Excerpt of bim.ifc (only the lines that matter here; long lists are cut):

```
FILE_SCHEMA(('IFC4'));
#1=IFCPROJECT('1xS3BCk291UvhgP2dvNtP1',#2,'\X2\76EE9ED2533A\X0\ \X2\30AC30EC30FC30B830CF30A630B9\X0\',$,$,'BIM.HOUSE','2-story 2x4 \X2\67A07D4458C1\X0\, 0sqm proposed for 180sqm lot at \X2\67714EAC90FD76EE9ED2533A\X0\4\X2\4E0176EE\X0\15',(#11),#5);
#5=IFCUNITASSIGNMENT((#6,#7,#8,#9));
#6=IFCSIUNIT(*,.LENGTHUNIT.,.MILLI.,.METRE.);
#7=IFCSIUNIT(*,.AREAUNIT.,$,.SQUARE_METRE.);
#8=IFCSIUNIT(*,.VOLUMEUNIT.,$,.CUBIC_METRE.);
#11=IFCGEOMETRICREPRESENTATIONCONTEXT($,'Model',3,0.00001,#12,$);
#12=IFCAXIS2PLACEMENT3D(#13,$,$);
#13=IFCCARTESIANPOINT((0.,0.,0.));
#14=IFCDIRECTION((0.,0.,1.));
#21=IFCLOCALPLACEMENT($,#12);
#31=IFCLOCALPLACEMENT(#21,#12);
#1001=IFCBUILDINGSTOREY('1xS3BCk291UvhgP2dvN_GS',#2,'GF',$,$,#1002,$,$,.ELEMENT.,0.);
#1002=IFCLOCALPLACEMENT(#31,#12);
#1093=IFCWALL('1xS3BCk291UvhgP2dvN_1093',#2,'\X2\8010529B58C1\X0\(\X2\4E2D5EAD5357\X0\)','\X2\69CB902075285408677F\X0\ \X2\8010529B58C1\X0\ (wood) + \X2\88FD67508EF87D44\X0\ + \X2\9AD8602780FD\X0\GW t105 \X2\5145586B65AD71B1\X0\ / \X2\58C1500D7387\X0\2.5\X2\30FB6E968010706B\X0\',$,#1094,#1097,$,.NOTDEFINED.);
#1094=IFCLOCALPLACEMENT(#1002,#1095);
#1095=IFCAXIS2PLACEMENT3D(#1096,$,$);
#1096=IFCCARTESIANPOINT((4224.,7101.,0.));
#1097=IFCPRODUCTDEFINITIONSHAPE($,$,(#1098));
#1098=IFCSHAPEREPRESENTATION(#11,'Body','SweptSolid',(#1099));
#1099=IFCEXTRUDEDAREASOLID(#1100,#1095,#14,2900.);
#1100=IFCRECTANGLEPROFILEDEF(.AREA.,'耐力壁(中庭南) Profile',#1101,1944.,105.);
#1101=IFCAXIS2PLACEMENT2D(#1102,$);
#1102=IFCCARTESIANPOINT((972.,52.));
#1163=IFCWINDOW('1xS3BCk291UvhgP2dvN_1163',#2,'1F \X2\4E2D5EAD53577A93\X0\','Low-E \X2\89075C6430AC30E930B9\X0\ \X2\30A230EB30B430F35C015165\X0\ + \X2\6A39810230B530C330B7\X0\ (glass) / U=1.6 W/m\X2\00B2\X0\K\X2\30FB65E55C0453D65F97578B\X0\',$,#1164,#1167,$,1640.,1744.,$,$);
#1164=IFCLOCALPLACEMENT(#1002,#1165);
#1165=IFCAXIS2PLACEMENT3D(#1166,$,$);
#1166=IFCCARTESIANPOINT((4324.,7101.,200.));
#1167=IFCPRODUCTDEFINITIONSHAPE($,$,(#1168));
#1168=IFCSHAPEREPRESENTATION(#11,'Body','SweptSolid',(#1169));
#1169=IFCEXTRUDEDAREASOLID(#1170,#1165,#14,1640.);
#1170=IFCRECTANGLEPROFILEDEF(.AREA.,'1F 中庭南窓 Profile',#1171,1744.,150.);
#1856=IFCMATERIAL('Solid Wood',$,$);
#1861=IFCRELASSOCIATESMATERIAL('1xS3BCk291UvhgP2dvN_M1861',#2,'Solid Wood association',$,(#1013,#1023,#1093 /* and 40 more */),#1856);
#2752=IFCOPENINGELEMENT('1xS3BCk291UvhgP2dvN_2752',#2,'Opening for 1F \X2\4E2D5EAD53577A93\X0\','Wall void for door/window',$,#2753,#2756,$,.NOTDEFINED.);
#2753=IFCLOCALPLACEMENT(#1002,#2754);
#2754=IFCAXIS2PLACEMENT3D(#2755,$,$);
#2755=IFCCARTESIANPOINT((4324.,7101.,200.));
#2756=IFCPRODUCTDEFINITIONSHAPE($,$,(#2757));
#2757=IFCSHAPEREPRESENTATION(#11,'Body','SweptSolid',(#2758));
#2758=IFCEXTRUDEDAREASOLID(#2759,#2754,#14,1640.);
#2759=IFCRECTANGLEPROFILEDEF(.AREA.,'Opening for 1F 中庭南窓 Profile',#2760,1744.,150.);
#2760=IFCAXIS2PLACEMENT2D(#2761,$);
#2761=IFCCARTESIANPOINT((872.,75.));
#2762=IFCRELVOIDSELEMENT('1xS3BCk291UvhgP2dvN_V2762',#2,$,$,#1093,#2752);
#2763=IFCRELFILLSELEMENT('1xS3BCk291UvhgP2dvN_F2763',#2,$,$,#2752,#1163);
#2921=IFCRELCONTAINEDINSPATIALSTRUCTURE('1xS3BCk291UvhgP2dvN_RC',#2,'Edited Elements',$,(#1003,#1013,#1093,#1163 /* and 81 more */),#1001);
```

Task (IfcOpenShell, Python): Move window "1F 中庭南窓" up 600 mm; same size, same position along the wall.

```python
import numpy as np
import ifcopenshell
import ifcopenshell.api.geometry
import ifcopenshell.util.placement
import ifcopenshell.util.unit

model = ifcopenshell.open("bim.ifc")
unit_scale = ifcopenshell.util.unit.calculate_unit_scale(model)

window = model.by_guid("1xS3BCk291UvhgP2dvN_1163")
opening = window.FillsVoids[0].RelatingOpeningElement
dz = 600.0

shift = np.array([0.0, 0.0, dz])
# The window is not placed relative to its opening, so move both.
for product in (opening, window):
    matrix = ifcopenshell.util.placement.get_local_placement(product.ObjectPlacement)
    matrix[:3, 3] += shift
    ifcopenshell.api.geometry.edit_object_placement(model, product=product, matrix=matrix, is_si=False)

print(f"moved by {dz * unit_scale:+.3f} m")

model.write("bim_edited.ifc")
```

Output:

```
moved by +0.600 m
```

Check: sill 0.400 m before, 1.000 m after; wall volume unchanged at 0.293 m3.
